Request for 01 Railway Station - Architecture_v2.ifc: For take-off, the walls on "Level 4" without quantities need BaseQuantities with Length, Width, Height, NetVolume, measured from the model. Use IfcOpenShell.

First a look at what the model holds.

```python
import ifcopenshell
import ifcopenshell.util.element
import ifcopenshell.util.unit

model = ifcopenshell.open("01 Railway Station - Architecture_v2.ifc")
print(model.schema)
for unit_type in ("LENGTHUNIT", "AREAUNIT", "VOLUMEUNIT"):
    print(unit_type, ifcopenshell.util.unit.calculate_unit_scale(model, unit_type))
storey = next(s for s in model.by_type("IfcBuildingStorey") if s.Name == "Level 4")
walls = [e for e in ifcopenshell.util.element.get_decomposition(storey) if e.is_a("IfcWall")]
for e in sorted(walls, key=lambda e: e.id()):
    print(e.id(), e.is_a(), e.Name, list(ifcopenshell.util.element.get_psets(e, qtos_only=True)), sep=" | ")
```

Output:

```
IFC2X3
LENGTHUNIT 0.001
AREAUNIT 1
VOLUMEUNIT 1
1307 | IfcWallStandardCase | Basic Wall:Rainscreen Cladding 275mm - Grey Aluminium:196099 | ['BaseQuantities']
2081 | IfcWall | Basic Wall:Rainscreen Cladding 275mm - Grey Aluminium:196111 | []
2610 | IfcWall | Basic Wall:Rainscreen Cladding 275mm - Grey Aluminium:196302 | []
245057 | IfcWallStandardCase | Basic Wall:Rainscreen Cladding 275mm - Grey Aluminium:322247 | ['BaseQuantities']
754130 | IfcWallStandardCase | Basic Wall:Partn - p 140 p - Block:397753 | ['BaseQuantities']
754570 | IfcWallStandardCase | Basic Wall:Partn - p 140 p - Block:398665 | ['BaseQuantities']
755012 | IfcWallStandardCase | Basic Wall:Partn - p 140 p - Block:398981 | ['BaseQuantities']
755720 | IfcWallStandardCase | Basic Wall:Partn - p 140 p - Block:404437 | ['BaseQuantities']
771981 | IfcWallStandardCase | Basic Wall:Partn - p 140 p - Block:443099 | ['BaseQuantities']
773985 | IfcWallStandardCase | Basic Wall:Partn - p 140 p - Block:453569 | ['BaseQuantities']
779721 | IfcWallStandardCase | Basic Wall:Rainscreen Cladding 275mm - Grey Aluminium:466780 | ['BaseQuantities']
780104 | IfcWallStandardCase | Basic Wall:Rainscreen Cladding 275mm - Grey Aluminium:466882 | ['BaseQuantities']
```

```python
import ifcopenshell
import ifcopenshell.api.pset
import ifcopenshell.geom
import ifcopenshell.util.element
import ifcopenshell.util.shape
import ifcopenshell.util.unit

model = ifcopenshell.open("01 Railway Station - Architecture_v2.ifc")
unit_scale = ifcopenshell.util.unit.calculate_unit_scale(model)
volume_scale = ifcopenshell.util.unit.calculate_unit_scale(model, "VOLUMEUNIT")
settings = ifcopenshell.geom.settings()

storey = next(s for s in model.by_type("IfcBuildingStorey") if s.Name == "Level 4")
walls = [e for e in ifcopenshell.util.element.get_decomposition(storey) if e.is_a("IfcWall")]

for e in sorted(walls, key=lambda e: e.id()):
    if ifcopenshell.util.element.get_psets(e, qtos_only=True, should_inherit=False):
        continue
    # Geometry comes back in metres, in the element's own axes.
    shape = ifcopenshell.geom.create_shape(settings, e)
    values = {
        "Length": ifcopenshell.util.shape.get_x(shape.geometry) / unit_scale,
        "Width": ifcopenshell.util.shape.get_y(shape.geometry) / unit_scale,
        "Height": ifcopenshell.util.shape.get_z(shape.geometry) / unit_scale,
        "NetVolume": ifcopenshell.util.shape.get_volume(shape.geometry) / volume_scale,
    }
    qto = ifcopenshell.api.pset.add_qto(model, product=e, name="BaseQuantities")
    ifcopenshell.api.pset.edit_qto(model, qto=qto, properties=values)
    print(e.id(), {k: round(v, 3) for k, v in values.items()})

model.write("01 Railway Station - Architecture_v2_updated.ifc")
```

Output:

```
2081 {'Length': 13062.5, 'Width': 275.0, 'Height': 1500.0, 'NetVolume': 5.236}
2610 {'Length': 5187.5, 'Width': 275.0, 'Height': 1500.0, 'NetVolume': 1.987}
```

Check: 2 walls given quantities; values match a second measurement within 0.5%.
